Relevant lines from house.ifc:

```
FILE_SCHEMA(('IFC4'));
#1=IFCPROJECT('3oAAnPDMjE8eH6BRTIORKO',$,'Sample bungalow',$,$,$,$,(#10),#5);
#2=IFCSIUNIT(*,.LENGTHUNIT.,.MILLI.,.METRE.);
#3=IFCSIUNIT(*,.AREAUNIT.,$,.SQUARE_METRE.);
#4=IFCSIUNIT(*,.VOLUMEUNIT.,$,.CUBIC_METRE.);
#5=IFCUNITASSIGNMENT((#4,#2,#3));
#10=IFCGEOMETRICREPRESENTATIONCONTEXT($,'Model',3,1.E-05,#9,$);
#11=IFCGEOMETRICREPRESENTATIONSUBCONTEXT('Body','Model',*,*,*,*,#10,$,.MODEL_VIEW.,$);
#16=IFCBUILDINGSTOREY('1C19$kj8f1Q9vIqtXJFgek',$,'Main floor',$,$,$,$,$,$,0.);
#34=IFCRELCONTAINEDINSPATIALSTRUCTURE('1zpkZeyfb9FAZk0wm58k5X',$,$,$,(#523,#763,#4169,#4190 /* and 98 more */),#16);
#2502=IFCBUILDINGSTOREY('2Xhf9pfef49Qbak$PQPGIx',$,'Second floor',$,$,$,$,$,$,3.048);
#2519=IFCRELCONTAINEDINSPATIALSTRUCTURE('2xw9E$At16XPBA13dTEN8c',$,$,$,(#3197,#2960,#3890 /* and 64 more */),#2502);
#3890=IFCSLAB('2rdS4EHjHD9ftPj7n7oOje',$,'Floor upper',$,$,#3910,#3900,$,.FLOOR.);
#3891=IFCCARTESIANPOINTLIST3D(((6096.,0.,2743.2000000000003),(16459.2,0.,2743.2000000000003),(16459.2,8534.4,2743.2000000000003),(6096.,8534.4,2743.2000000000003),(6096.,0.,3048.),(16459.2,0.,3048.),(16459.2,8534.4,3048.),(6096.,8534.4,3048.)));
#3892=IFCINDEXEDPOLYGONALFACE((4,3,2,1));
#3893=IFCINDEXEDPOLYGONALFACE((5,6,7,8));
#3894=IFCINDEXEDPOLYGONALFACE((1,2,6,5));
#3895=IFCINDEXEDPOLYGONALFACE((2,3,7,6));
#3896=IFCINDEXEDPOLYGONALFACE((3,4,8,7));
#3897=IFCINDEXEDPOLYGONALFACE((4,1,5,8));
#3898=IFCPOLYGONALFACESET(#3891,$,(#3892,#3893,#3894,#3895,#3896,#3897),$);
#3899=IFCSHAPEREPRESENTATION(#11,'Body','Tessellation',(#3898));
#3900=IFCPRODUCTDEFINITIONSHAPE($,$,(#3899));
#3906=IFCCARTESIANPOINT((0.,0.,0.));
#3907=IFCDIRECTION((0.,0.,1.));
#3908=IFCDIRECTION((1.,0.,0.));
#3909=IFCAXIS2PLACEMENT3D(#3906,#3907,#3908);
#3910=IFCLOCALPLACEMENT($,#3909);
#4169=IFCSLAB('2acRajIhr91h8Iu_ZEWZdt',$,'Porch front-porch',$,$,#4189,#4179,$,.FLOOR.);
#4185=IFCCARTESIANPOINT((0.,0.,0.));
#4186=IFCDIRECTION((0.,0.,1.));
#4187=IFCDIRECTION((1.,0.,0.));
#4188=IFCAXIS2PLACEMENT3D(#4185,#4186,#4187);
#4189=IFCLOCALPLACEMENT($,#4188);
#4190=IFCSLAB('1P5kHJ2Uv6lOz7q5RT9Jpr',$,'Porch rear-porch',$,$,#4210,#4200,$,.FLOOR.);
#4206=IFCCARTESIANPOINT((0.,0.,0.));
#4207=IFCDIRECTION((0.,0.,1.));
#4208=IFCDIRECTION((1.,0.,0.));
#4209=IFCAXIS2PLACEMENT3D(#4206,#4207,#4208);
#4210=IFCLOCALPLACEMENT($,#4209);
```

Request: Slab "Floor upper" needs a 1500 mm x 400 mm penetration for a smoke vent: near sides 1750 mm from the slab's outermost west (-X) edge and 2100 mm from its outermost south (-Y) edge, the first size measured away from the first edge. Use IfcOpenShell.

```python
import numpy as np
import ifcopenshell
import ifcopenshell.api.feature
import ifcopenshell.api.geometry
import ifcopenshell.api.root
import ifcopenshell.geom
import ifcopenshell.util.placement
import ifcopenshell.util.representation
import ifcopenshell.util.shape
import ifcopenshell.util.unit

model = ifcopenshell.open("house.ifc")
unit_scale = ifcopenshell.util.unit.calculate_unit_scale(model)
settings = ifcopenshell.geom.settings()


def volume(element):
    """Net volume in cubic metres, openings subtracted."""
    shape = ifcopenshell.geom.create_shape(settings, element)
    return ifcopenshell.util.shape.get_volume(shape.geometry)


slab = model.by_guid("2rdS4EHjHD9ftPj7n7oOje")
before = volume(slab)

# Extent in the slab's own axes, in metres. The edges named are its -X and -Y sides.
slab_shape = ifcopenshell.geom.create_shape(settings, slab)
vertices = ifcopenshell.util.shape.get_vertices(slab_shape.geometry)
x_min, y_min, bottom = vertices.min(axis=0)
top = vertices[:, 2].max()

opening = ifcopenshell.api.root.create_entity(model, ifc_class="IfcOpeningElement", name="Smoke vent opening", predefined_type="OPENING")
context = ifcopenshell.util.representation.get_context(model, "Model", "Body", "MODEL_VIEW")
width, depth = 1.5, 0.4
outline = [(0.0, 0.0), (width, 0.0), (width, depth), (0.0, depth), (0.0, 0.0)]
# Overshoot both faces by 50 mm so the cut is clean.
shape = ifcopenshell.api.geometry.add_slab_representation(
    model, context=context, depth=top - bottom + 0.1, polyline=outline
)
ifcopenshell.api.geometry.assign_representation(model, product=opening, representation=shape)

matrix = ifcopenshell.util.placement.get_local_placement(slab.ObjectPlacement)
matrix[:, 3] = matrix @ np.append(np.array([x_min + 1.75, y_min + 2.1, bottom - 0.05]) / unit_scale, 1.0)
ifcopenshell.api.geometry.edit_object_placement(model, product=opening, matrix=matrix, is_si=False)
ifcopenshell.api.feature.add_feature(model, feature=opening, element=slab)

after = volume(slab)

print(f"slab volume {before:.3f} -> {after:.3f} m3")

model.write("house_edited.ifc")
```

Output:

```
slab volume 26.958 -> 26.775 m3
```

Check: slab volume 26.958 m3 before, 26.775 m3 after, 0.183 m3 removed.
